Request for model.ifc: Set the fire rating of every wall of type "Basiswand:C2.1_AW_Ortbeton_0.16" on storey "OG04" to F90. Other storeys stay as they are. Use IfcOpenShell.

First a look at what the model holds.

```python
import ifcopenshell
import ifcopenshell.util.element

model = ifcopenshell.open("model.ifc")
print(model.schema)
storey = next(s for s in model.by_type("IfcBuildingStorey") if s.Name == "OG04")
walls = [e for e in ifcopenshell.util.element.get_decomposition(storey) if e.is_a("IfcWall")]
seen = {}
for e in walls:
    element_type = ifcopenshell.util.element.get_type(e)
    key = (element_type.Name if element_type != e and element_type else None, ifcopenshell.util.element.get_pset(e, "Pset_WallCommon", "FireRating"))
    seen[key] = seen.get(key, 0) + 1
for (name, value), count in sorted(seen.items(), key=str):
    print(count, "x", name, "|", value)
```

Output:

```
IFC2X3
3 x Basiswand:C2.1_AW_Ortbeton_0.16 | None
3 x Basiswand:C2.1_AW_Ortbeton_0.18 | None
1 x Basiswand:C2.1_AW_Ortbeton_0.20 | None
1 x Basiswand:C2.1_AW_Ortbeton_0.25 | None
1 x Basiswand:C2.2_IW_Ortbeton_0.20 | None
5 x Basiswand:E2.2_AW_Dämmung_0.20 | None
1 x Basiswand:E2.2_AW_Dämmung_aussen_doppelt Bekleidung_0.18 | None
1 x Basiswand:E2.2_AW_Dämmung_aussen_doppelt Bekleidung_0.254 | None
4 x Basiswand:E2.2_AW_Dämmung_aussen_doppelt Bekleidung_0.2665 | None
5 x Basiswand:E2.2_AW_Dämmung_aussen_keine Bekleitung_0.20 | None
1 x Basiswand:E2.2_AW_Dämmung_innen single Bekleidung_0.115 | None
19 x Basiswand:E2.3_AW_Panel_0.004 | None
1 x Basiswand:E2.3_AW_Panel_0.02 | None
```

```python
import ifcopenshell
import ifcopenshell.api.pset
import ifcopenshell.util.element

model = ifcopenshell.open("model.ifc")

storey = next(s for s in model.by_type("IfcBuildingStorey") if s.Name == "OG04")
walls = [e for e in ifcopenshell.util.element.get_decomposition(storey) if e.is_a("IfcWall")]

count = 0
for e in walls:
    element_type = ifcopenshell.util.element.get_type(e)
    if element_type in (None, e) or element_type.Name != "Basiswand:C2.1_AW_Ortbeton_0.16":
        continue
    # add_pset returns the element's existing set when there is one.
    pset = ifcopenshell.api.pset.add_pset(model, product=e, name="Pset_WallCommon")
    ifcopenshell.api.pset.edit_pset(model, pset=pset, properties={"FireRating": "F90"})
    count += 1

print(count, "walls updated")

model.write("model_edited.ifc")
```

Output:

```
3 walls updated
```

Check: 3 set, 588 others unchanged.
